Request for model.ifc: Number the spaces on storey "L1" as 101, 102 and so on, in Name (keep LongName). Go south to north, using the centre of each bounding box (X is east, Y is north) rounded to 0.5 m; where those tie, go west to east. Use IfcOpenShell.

First a look at what the model holds.

```python
import ifcopenshell
import ifcopenshell.util.element
import ifcopenshell.util.placement

model = ifcopenshell.open("model.ifc")
print(model.schema)
storey = next(s for s in model.by_type("IfcBuildingStorey") if s.Name == "L1")
spaces = [e for e in ifcopenshell.util.element.get_decomposition(storey) if e.is_a("IfcSpace")]
for e in sorted(spaces, key=lambda e: e.id()):
    origin = ifcopenshell.util.placement.get_local_placement(e.ObjectPlacement)[:3, 3]
    print(e.id(), e.Name, e.LongName, origin.round(2) + 0.0, sep=" | ")
```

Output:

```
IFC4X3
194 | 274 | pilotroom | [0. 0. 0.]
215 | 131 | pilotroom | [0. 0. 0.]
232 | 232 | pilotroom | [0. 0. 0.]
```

```python
import ifcopenshell
import ifcopenshell.geom
import ifcopenshell.util.element
import ifcopenshell.util.shape

model = ifcopenshell.open("model.ifc")
settings = ifcopenshell.geom.settings()
settings.set("use-world-coords", True)


def centre(element):
    shape = ifcopenshell.geom.create_shape(settings, element)
    return ifcopenshell.util.shape.get_bbox_centroid(shape.geometry)


storey = next(s for s in model.by_type("IfcBuildingStorey") if s.Name == "L1")
spaces = [e for e in ifcopenshell.util.element.get_decomposition(storey) if e.is_a("IfcSpace")]

# Insertion points can sit at a corner or the storey origin, so sort by the geometry (in metres).
centres = {e: centre(e) for e in spaces}
spaces.sort(key=lambda e: (round(centres[e][1] / 0.5), centres[e][0]))

for i, e in enumerate(spaces, start=1):
    number = f"1{i:02d}"
    e.Name = number
    print(e.id(), number)

model.write("model_updated.ifc")
```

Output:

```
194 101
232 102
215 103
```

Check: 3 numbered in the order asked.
